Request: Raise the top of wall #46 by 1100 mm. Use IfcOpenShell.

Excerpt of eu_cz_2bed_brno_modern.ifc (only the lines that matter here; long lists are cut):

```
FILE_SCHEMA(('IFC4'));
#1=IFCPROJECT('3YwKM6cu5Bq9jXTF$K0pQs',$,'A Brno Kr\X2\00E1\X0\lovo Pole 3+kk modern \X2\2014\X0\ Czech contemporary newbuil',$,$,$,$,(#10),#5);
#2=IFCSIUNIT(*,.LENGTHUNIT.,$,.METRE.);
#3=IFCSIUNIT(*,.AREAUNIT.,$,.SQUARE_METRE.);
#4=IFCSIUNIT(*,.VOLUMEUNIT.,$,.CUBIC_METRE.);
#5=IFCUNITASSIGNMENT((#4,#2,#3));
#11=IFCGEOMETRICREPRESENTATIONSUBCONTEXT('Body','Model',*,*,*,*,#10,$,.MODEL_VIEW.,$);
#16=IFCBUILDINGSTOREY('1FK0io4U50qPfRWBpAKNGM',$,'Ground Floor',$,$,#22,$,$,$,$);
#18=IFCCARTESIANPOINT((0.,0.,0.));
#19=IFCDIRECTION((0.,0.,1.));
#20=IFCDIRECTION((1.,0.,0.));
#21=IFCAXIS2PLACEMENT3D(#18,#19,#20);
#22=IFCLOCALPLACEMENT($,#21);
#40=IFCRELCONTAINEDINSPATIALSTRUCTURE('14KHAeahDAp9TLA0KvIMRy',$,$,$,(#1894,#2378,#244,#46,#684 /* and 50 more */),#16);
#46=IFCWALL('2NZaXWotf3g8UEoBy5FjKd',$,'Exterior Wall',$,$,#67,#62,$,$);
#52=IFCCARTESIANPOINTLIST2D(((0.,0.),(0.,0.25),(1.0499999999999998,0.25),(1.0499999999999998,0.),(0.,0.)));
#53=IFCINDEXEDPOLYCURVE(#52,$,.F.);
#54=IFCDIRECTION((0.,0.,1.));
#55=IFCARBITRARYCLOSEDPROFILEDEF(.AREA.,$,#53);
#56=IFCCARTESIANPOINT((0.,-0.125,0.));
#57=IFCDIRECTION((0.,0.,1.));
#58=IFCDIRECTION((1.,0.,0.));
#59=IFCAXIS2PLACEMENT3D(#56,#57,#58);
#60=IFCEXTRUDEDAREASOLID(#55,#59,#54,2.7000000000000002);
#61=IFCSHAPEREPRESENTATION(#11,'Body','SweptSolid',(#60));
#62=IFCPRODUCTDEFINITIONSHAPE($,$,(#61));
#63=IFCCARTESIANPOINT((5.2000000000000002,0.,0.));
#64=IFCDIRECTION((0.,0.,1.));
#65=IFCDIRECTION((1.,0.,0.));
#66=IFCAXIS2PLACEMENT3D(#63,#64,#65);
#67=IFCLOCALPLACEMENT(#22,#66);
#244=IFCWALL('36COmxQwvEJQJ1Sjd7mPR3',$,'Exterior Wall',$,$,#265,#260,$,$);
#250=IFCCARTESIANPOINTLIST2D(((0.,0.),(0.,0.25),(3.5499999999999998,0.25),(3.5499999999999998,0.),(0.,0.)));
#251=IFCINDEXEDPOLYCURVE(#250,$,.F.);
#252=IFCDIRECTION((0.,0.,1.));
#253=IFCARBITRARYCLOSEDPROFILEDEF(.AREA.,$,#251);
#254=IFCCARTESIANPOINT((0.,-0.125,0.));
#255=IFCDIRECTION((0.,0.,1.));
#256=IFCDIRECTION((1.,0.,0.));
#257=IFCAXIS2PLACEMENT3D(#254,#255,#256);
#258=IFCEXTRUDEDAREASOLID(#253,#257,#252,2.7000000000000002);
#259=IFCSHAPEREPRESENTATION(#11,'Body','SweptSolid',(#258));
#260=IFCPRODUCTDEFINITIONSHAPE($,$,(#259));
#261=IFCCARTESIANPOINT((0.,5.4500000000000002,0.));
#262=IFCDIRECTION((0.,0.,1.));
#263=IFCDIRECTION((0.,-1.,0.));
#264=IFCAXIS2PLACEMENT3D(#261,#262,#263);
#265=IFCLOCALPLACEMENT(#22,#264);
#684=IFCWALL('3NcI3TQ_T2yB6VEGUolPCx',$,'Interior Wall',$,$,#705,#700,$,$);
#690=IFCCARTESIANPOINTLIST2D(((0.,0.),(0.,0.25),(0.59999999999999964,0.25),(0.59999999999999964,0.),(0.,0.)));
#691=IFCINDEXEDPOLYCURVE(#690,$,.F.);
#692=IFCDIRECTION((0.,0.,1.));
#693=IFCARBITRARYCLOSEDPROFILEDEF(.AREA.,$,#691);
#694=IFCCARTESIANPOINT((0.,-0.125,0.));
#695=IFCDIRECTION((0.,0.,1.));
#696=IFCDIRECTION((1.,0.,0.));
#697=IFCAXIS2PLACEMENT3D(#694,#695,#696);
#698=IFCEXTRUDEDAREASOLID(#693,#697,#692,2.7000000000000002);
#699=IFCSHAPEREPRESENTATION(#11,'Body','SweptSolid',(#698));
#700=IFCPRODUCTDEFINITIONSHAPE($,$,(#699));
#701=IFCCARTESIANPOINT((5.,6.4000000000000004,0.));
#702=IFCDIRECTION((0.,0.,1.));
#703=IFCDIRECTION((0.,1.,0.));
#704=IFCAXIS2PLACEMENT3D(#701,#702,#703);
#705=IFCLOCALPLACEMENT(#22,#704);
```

```python
import ifcopenshell
import ifcopenshell.geom
import ifcopenshell.util.representation
import ifcopenshell.util.shape
import ifcopenshell.util.unit

model = ifcopenshell.open("eu_cz_2bed_brno_modern.ifc")
unit_scale = ifcopenshell.util.unit.calculate_unit_scale(model)
settings = ifcopenshell.geom.settings()


def volume(element):
    """Net volume in cubic metres, openings subtracted."""
    shape = ifcopenshell.geom.create_shape(settings, element)
    return ifcopenshell.util.shape.get_volume(shape.geometry)


wall = model.by_guid("2NZaXWotf3g8UEoBy5FjKd")
before = volume(wall)

body = ifcopenshell.util.representation.get_representation(wall, "Model", "Body")
solid = body.Items[0]
old_height = solid.Depth
solid.Depth += 1.1 / unit_scale
after = volume(wall)

print(f"height {old_height:g} -> {solid.Depth:g}, volume {before:.3f} -> {after:.3f} m3")

model.write("eu_cz_2bed_brno_modern_v2.ifc")
```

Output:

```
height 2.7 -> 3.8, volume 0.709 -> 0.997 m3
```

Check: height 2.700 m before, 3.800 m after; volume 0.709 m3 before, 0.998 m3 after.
